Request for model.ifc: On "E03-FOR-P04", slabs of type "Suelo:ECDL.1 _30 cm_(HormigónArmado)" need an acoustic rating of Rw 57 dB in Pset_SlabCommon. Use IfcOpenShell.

First a look at what the model holds.

```python
import ifcopenshell
import ifcopenshell.util.element

model = ifcopenshell.open("model.ifc")
print(model.schema)
storey = next(s for s in model.by_type("IfcBuildingStorey") if s.Name == "E03-FOR-P04")
slabs = [e for e in ifcopenshell.util.element.get_decomposition(storey) if e.is_a("IfcSlab")]
seen = {}
for e in slabs:
    element_type = ifcopenshell.util.element.get_type(e)
    key = (element_type.Name if element_type != e and element_type else None, ifcopenshell.util.element.get_pset(e, "Pset_SlabCommon", "AcousticRating"))
    seen[key] = seen.get(key, 0) + 1
for (name, value), count in sorted(seen.items(), key=str):
    print(count, "x", name, "|", value)
```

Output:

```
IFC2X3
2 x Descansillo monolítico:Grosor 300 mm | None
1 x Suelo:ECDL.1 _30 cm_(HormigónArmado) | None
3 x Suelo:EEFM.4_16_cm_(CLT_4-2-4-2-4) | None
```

```python
import ifcopenshell
import ifcopenshell.api.pset
import ifcopenshell.util.element

model = ifcopenshell.open("model.ifc")

storey = next(s for s in model.by_type("IfcBuildingStorey") if s.Name == "E03-FOR-P04")
slabs = [e for e in ifcopenshell.util.element.get_decomposition(storey) if e.is_a("IfcSlab")]

count = 0
for e in slabs:
    element_type = ifcopenshell.util.element.get_type(e)
    if element_type in (None, e) or element_type.Name != "Suelo:ECDL.1 _30 cm_(HormigónArmado)":
        continue
    # add_pset returns the element's existing set when there is one.
    pset = ifcopenshell.api.pset.add_pset(model, product=e, name="Pset_SlabCommon")
    ifcopenshell.api.pset.edit_pset(model, pset=pset, properties={"AcousticRating": "Rw 57 dB"})
    count += 1

print(count, "slabs updated")

model.write("model_v2.ifc")
```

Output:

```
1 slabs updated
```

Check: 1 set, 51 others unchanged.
